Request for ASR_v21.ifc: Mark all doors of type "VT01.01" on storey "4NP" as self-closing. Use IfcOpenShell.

First a look at what the model holds.

```python
import ifcopenshell
import ifcopenshell.util.element

model = ifcopenshell.open("ASR_v21.ifc")
print(model.schema)
storey = next(s for s in model.by_type("IfcBuildingStorey") if s.Name == "4NP")
doors = [e for e in ifcopenshell.util.element.get_decomposition(storey) if e.is_a("IfcDoor")]
seen = {}
for e in doors:
    element_type = ifcopenshell.util.element.get_type(e)
    key = (element_type.Name if element_type != e and element_type else None, ifcopenshell.util.element.get_pset(e, "Pset_DoorCommon", "SelfClosing"))
    seen[key] = seen.get(key, 0) + 1
for (name, value), count in sorted(seen.items(), key=str):
    print(count, "x", name, "|", value)
```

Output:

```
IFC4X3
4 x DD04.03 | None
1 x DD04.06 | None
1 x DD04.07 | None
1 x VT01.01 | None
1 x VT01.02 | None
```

```python
import ifcopenshell
import ifcopenshell.api.pset
import ifcopenshell.util.element

model = ifcopenshell.open("ASR_v21.ifc")

storey = next(s for s in model.by_type("IfcBuildingStorey") if s.Name == "4NP")
doors = [e for e in ifcopenshell.util.element.get_decomposition(storey) if e.is_a("IfcDoor")]

count = 0
for e in doors:
    element_type = ifcopenshell.util.element.get_type(e)
    if element_type in (None, e) or element_type.Name != "VT01.01":
        continue
    # add_pset returns the element's existing set when there is one.
    pset = ifcopenshell.api.pset.add_pset(model, product=e, name="Pset_DoorCommon")
    ifcopenshell.api.pset.edit_pset(model, pset=pset, properties={"SelfClosing": True})
    count += 1

print(count, "doors updated")

model.write("ASR_v21_v2.ifc")
```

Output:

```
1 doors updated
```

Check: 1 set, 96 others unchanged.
